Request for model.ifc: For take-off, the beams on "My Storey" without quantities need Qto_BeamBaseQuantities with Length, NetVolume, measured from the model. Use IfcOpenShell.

First a look at what the model holds.

```python
import ifcopenshell
import ifcopenshell.util.element
import ifcopenshell.util.unit

model = ifcopenshell.open("model.ifc")
print(model.schema)
for unit_type in ("LENGTHUNIT", "AREAUNIT", "VOLUMEUNIT"):
    print(unit_type, ifcopenshell.util.unit.calculate_unit_scale(model, unit_type))
storey = next(s for s in model.by_type("IfcBuildingStorey") if s.Name == "My Storey")
beams = [e for e in ifcopenshell.util.element.get_decomposition(storey) if e.is_a("IfcBeam")]
for e in sorted(beams, key=lambda e: e.id()):
    print(e.id(), e.is_a(), e.Name, list(ifcopenshell.util.element.get_psets(e, qtos_only=True)), sep=" | ")
```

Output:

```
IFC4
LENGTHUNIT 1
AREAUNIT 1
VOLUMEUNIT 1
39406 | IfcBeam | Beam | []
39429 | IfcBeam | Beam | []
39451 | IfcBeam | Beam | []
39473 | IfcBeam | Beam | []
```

```python
import ifcopenshell
import ifcopenshell.api.pset
import ifcopenshell.geom
import ifcopenshell.util.element
import ifcopenshell.util.shape
import ifcopenshell.util.unit

model = ifcopenshell.open("model.ifc")
unit_scale = ifcopenshell.util.unit.calculate_unit_scale(model)
volume_scale = ifcopenshell.util.unit.calculate_unit_scale(model, "VOLUMEUNIT")
settings = ifcopenshell.geom.settings()

storey = next(s for s in model.by_type("IfcBuildingStorey") if s.Name == "My Storey")
beams = [e for e in ifcopenshell.util.element.get_decomposition(storey) if e.is_a("IfcBeam")]

for e in sorted(beams, key=lambda e: e.id()):
    if ifcopenshell.util.element.get_psets(e, qtos_only=True, should_inherit=False):
        continue
    # Geometry comes back in metres, in the element's own axes.
    shape = ifcopenshell.geom.create_shape(settings, e)
    values = {
        "Length": ifcopenshell.util.shape.get_max_xyz(shape.geometry) / unit_scale,
        "NetVolume": ifcopenshell.util.shape.get_volume(shape.geometry) / volume_scale,
    }
    qto = ifcopenshell.api.pset.add_qto(model, product=e, name="Qto_BeamBaseQuantities")
    ifcopenshell.api.pset.edit_qto(model, qto=qto, properties=values)
    print(e.id(), {k: round(v, 3) for k, v in values.items()})

model.write("model_updated.ifc")
```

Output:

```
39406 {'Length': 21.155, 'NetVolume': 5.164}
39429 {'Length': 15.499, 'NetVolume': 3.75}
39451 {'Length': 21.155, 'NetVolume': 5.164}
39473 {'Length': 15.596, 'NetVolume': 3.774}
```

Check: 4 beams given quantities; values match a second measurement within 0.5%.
